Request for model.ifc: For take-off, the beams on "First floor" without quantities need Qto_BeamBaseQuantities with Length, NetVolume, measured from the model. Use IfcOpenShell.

First a look at what the model holds.

```python
import ifcopenshell
import ifcopenshell.util.element
import ifcopenshell.util.unit

model = ifcopenshell.open("model.ifc")
print(model.schema)
for unit_type in ("LENGTHUNIT", "AREAUNIT", "VOLUMEUNIT"):
    print(unit_type, ifcopenshell.util.unit.calculate_unit_scale(model, unit_type))
storey = next(s for s in model.by_type("IfcBuildingStorey") if s.Name == "First floor")
beams = [e for e in ifcopenshell.util.element.get_decomposition(storey) if e.is_a("IfcBeam")]
for e in sorted(beams, key=lambda e: e.id()):
    print(e.id(), e.is_a(), e.Name, list(ifcopenshell.util.element.get_psets(e, qtos_only=True)), sep=" | ")
```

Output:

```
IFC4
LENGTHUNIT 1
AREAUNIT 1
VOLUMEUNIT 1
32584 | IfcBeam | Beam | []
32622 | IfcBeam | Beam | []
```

```python
import ifcopenshell
import ifcopenshell.api.pset
import ifcopenshell.geom
import ifcopenshell.util.element
import ifcopenshell.util.shape
import ifcopenshell.util.unit

model = ifcopenshell.open("model.ifc")
unit_scale = ifcopenshell.util.unit.calculate_unit_scale(model)
volume_scale = ifcopenshell.util.unit.calculate_unit_scale(model, "VOLUMEUNIT")
settings = ifcopenshell.geom.settings()

storey = next(s for s in model.by_type("IfcBuildingStorey") if s.Name == "First floor")
beams = [e for e in ifcopenshell.util.element.get_decomposition(storey) if e.is_a("IfcBeam")]

for e in sorted(beams, key=lambda e: e.id()):
    if ifcopenshell.util.element.get_psets(e, qtos_only=True, should_inherit=False):
        continue
    # Geometry comes back in metres, in the element's own axes.
    shape = ifcopenshell.geom.create_shape(settings, e)
    values = {
        "Length": ifcopenshell.util.shape.get_max_xyz(shape.geometry) / unit_scale,
        "NetVolume": ifcopenshell.util.shape.get_volume(shape.geometry) / volume_scale,
    }
    qto = ifcopenshell.api.pset.add_qto(model, product=e, name="Qto_BeamBaseQuantities")
    ifcopenshell.api.pset.edit_qto(model, qto=qto, properties=values)
    print(e.id(), {k: round(v, 3) for k, v in values.items()})

model.write("model_rev.ifc")
```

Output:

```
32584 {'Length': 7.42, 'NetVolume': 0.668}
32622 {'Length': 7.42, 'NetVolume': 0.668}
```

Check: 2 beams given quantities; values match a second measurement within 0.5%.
